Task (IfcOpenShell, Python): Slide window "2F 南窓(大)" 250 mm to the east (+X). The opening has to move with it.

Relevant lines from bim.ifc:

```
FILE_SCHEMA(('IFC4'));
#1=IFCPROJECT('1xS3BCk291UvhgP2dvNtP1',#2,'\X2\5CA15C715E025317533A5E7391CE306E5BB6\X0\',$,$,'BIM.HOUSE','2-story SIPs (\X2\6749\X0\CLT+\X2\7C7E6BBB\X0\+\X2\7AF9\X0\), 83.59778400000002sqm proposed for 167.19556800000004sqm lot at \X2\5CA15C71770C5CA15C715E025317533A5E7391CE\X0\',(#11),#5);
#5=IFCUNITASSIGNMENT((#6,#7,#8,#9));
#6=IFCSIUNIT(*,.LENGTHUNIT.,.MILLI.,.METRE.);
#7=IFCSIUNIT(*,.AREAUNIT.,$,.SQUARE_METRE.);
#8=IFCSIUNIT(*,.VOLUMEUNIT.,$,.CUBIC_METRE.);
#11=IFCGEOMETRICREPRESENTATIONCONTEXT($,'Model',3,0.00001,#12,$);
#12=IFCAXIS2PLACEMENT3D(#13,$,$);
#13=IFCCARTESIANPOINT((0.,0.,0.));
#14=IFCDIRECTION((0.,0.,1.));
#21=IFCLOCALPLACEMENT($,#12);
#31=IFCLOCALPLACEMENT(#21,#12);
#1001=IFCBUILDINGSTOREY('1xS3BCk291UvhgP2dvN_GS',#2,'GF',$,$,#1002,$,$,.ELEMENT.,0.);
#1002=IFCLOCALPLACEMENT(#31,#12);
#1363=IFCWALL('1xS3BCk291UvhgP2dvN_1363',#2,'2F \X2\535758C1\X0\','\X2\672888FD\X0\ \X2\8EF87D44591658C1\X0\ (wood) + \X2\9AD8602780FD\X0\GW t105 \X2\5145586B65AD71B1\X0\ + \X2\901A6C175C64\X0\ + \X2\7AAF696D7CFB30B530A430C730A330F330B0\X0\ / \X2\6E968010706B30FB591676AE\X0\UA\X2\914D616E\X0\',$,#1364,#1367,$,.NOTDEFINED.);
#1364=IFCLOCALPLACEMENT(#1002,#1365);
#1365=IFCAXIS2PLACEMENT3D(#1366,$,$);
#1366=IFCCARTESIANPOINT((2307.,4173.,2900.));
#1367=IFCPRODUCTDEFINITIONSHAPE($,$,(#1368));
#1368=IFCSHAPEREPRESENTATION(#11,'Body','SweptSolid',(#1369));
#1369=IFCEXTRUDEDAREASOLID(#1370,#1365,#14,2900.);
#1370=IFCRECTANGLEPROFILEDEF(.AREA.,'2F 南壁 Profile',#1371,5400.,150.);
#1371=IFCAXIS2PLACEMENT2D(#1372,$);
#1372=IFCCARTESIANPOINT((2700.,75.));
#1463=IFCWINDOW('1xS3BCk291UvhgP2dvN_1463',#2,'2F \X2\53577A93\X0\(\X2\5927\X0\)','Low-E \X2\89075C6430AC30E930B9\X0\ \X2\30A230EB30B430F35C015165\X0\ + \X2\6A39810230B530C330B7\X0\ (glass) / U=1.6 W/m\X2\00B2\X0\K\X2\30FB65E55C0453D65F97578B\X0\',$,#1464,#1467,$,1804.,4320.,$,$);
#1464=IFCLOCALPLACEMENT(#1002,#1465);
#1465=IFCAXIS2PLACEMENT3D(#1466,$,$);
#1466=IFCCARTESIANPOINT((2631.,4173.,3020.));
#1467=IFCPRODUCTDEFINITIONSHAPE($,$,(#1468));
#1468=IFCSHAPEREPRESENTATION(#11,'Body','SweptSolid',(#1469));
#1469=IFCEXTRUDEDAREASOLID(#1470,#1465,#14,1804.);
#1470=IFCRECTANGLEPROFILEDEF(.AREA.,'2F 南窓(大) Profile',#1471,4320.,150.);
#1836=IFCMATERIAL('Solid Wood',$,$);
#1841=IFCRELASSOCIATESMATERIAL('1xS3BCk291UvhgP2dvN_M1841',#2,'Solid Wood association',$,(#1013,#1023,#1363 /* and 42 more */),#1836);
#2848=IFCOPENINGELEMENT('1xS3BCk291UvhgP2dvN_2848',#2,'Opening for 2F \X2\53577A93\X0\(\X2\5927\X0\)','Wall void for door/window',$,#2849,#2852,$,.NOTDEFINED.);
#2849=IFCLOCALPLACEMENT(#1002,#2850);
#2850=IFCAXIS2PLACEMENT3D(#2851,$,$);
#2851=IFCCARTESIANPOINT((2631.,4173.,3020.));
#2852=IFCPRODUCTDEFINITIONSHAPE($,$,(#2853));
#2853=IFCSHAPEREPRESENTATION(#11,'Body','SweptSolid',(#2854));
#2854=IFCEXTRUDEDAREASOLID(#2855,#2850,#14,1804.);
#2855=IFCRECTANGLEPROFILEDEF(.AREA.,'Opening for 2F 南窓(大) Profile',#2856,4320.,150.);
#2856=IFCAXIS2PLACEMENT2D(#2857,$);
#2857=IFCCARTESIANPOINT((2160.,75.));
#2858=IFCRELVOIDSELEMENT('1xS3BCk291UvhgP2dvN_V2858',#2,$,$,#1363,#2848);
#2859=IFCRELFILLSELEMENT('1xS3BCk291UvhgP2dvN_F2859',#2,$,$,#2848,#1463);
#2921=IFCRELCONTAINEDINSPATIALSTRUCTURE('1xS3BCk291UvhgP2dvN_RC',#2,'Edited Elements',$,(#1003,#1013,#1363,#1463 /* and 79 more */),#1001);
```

```python
import ifcopenshell
import ifcopenshell.api.geometry
import ifcopenshell.util.placement

model = ifcopenshell.open("bim.ifc")

window = model.by_guid("1xS3BCk291UvhgP2dvN_1463")
opening = window.FillsVoids[0].RelatingOpeningElement
wall = opening.VoidsElements[0].RelatingBuildingElement

wall_matrix = ifcopenshell.util.placement.get_local_placement(wall.ObjectPlacement)
shift = wall_matrix[:3, 0] * 250.0
before = ifcopenshell.util.placement.get_local_placement(window.ObjectPlacement)[:3, 3].copy()

# The window is not placed relative to its opening, so move both.
for product in (opening, window):
    matrix = ifcopenshell.util.placement.get_local_placement(product.ObjectPlacement)
    matrix[:3, 3] += shift
    ifcopenshell.api.geometry.edit_object_placement(model, product=product, matrix=matrix, is_si=False)

after = ifcopenshell.util.placement.get_local_placement(window.ObjectPlacement)[:3, 3]
print("window moved by", (after - before).round(3) + 0.0)

model.write("bim_rev.ifc")
```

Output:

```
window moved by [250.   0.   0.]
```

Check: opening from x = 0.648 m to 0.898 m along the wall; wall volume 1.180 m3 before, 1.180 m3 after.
